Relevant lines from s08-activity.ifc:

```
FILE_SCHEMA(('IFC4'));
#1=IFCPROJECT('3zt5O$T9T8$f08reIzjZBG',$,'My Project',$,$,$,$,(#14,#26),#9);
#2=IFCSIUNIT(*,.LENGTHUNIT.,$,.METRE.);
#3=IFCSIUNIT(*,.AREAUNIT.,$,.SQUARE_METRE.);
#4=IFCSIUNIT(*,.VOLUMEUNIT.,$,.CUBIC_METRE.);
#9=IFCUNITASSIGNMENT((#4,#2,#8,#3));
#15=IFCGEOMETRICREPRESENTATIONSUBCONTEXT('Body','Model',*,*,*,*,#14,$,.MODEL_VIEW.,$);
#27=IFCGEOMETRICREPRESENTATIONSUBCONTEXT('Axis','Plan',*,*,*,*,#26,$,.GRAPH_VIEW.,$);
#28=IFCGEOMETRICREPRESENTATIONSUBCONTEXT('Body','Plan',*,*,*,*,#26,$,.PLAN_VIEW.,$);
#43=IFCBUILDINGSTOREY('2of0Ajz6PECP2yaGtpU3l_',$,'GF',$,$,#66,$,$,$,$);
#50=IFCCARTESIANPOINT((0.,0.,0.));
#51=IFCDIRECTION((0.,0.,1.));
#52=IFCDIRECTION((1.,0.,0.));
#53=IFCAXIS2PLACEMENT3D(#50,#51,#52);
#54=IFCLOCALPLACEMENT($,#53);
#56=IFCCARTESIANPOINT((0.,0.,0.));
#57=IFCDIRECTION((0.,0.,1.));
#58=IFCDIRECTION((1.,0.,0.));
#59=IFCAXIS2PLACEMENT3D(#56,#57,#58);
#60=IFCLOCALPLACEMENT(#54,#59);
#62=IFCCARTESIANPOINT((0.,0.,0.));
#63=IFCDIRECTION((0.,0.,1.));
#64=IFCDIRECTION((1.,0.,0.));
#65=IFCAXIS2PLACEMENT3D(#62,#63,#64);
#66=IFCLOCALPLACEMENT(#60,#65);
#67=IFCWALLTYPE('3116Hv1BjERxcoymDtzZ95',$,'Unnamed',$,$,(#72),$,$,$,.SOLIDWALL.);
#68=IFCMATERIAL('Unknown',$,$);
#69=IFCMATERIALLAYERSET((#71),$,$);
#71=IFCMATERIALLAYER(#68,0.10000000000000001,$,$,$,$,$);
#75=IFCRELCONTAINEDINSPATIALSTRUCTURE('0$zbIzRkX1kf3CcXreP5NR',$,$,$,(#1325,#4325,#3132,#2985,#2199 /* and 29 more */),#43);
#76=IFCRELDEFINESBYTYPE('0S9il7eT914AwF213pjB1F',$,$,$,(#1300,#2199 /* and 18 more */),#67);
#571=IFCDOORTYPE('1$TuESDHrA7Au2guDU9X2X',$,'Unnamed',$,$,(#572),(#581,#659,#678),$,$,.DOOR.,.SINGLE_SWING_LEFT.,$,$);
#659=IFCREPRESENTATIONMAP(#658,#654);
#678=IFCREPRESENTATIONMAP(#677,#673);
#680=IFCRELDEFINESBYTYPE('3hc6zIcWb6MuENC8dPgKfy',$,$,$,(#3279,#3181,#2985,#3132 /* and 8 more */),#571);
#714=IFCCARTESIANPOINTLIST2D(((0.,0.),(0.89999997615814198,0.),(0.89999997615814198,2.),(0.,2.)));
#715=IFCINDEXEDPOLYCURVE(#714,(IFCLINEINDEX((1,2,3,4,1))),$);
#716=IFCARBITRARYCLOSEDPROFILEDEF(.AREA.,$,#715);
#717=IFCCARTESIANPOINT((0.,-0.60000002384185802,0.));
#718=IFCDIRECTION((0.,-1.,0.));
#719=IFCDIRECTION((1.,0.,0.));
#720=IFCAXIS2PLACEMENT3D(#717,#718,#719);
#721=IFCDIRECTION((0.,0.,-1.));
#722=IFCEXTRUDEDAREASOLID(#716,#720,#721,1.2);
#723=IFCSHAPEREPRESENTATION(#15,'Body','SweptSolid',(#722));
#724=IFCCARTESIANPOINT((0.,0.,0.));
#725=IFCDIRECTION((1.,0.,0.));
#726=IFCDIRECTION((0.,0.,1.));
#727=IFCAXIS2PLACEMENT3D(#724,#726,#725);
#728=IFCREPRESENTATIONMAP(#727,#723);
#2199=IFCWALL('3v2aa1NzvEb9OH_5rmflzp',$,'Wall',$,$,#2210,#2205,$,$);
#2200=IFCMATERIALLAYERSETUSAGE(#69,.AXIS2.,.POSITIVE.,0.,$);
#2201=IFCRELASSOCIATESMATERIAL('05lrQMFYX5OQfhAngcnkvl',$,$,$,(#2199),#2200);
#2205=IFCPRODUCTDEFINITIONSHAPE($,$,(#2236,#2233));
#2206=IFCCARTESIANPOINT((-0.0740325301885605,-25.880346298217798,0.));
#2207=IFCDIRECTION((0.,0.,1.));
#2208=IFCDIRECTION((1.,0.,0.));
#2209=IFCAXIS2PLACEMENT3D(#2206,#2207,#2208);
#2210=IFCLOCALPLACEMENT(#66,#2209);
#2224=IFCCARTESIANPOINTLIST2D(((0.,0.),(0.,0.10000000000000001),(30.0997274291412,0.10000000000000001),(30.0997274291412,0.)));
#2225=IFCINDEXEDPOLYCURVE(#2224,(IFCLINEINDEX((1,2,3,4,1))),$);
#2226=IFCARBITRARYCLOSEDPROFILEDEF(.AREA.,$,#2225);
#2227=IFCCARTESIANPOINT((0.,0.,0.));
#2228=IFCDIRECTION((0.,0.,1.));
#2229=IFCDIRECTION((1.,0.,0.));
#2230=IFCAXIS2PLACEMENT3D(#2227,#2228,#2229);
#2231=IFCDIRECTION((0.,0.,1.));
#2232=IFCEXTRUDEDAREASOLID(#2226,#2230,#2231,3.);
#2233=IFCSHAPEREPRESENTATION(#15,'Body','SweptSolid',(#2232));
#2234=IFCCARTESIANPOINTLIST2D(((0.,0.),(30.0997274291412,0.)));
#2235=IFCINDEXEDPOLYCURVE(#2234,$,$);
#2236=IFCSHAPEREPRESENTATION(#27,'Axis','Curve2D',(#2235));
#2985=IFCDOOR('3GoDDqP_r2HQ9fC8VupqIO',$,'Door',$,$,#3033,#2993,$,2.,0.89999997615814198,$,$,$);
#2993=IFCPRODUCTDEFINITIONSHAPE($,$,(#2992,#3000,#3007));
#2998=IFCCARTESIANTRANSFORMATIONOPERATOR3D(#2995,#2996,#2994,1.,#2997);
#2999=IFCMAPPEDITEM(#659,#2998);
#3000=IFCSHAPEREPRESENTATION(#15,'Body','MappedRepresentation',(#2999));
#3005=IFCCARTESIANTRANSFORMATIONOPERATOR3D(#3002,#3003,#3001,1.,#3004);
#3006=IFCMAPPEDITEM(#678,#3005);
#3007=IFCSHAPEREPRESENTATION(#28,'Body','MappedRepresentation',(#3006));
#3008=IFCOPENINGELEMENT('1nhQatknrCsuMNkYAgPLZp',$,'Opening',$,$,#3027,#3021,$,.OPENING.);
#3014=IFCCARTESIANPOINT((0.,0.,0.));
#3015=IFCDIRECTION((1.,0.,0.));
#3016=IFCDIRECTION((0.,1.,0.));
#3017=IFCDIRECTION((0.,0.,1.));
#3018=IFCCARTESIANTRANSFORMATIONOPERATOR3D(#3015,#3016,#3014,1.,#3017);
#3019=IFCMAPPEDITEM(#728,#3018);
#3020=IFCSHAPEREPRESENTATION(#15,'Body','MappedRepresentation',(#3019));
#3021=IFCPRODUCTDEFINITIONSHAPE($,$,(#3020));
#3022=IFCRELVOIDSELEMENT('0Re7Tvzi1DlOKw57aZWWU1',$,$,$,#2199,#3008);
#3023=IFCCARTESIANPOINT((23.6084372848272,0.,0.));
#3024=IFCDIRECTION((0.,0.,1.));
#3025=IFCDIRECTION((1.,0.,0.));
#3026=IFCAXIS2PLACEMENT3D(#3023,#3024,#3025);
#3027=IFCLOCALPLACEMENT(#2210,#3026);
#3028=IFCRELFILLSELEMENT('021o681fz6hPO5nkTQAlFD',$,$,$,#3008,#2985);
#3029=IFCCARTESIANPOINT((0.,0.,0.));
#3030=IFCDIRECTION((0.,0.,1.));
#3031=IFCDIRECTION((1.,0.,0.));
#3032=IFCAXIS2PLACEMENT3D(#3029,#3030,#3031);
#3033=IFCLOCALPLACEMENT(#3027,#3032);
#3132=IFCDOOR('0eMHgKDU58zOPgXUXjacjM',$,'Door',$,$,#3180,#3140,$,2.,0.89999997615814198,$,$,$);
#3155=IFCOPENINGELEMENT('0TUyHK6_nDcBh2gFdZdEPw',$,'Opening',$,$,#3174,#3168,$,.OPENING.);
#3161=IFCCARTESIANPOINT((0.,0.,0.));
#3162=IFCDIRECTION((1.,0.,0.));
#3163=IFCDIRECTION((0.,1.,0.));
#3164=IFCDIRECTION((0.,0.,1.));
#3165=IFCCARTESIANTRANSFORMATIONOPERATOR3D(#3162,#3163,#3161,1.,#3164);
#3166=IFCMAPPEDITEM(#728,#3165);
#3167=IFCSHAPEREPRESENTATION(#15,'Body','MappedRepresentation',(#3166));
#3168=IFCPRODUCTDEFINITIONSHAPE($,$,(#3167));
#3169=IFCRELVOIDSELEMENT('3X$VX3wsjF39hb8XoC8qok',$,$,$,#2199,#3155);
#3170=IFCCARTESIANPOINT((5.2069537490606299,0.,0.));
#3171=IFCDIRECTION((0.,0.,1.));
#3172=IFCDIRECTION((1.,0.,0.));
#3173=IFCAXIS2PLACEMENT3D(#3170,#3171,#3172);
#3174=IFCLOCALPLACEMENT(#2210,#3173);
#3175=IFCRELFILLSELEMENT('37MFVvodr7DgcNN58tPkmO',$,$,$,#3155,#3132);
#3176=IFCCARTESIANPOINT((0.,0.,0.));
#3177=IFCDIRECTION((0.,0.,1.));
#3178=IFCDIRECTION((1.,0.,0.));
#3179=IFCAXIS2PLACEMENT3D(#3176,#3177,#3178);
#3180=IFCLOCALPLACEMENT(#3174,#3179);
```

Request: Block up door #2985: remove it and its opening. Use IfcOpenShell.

```python
import ifcopenshell
import ifcopenshell.api.feature
import ifcopenshell.api.root
import ifcopenshell.geom
import ifcopenshell.util.shape

model = ifcopenshell.open("s08-activity.ifc")
settings = ifcopenshell.geom.settings()


def volume(element):
    """Net volume in cubic metres, openings subtracted."""
    shape = ifcopenshell.geom.create_shape(settings, element)
    return ifcopenshell.util.shape.get_volume(shape.geometry)


door = model.by_id(2985)
opening = door.FillsVoids[0].RelatingOpeningElement
wall = opening.VoidsElements[0].RelatingBuildingElement
before = volume(wall)

ifcopenshell.api.root.remove_product(model, product=door)
ifcopenshell.api.feature.remove_feature(model, feature=opening)

after = volume(wall)

print(f"wall volume {before:.3f} -> {after:.3f} m3")

model.write("s08-activity_edited.ifc")
```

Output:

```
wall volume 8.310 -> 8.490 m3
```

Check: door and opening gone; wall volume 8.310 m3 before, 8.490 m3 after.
